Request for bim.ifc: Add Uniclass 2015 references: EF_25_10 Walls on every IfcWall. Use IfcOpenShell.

First a look at what the model holds.

```python
import ifcopenshell

model = ifcopenshell.open("bim.ifc")
print(model.schema)
print("classifications:", [c.Name for c in model.by_type("IfcClassification")])
for ifc_class in ("IfcDoor", "IfcRoof", "IfcStair", "IfcWall", "IfcWindow"):
    print(ifc_class, len(model.by_type(ifc_class)))
```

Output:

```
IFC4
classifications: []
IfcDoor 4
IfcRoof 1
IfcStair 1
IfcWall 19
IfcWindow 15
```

```python
import ifcopenshell
import ifcopenshell.api.classification

model = ifcopenshell.open("bim.ifc")

system = ifcopenshell.api.classification.add_classification(model, classification="Uniclass 2015")

codes = {
    "IfcWall": ("EF_25_10", "Walls"),
}
for ifc_class, (code, name) in codes.items():
    products = model.by_type(ifc_class)
    ifcopenshell.api.classification.add_reference(
        model, products=products, classification=system, identification=code, name=name
    )
    print(code, len(products))

model.write("bim_updated.ifc")
```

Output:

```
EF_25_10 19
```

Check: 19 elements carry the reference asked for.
